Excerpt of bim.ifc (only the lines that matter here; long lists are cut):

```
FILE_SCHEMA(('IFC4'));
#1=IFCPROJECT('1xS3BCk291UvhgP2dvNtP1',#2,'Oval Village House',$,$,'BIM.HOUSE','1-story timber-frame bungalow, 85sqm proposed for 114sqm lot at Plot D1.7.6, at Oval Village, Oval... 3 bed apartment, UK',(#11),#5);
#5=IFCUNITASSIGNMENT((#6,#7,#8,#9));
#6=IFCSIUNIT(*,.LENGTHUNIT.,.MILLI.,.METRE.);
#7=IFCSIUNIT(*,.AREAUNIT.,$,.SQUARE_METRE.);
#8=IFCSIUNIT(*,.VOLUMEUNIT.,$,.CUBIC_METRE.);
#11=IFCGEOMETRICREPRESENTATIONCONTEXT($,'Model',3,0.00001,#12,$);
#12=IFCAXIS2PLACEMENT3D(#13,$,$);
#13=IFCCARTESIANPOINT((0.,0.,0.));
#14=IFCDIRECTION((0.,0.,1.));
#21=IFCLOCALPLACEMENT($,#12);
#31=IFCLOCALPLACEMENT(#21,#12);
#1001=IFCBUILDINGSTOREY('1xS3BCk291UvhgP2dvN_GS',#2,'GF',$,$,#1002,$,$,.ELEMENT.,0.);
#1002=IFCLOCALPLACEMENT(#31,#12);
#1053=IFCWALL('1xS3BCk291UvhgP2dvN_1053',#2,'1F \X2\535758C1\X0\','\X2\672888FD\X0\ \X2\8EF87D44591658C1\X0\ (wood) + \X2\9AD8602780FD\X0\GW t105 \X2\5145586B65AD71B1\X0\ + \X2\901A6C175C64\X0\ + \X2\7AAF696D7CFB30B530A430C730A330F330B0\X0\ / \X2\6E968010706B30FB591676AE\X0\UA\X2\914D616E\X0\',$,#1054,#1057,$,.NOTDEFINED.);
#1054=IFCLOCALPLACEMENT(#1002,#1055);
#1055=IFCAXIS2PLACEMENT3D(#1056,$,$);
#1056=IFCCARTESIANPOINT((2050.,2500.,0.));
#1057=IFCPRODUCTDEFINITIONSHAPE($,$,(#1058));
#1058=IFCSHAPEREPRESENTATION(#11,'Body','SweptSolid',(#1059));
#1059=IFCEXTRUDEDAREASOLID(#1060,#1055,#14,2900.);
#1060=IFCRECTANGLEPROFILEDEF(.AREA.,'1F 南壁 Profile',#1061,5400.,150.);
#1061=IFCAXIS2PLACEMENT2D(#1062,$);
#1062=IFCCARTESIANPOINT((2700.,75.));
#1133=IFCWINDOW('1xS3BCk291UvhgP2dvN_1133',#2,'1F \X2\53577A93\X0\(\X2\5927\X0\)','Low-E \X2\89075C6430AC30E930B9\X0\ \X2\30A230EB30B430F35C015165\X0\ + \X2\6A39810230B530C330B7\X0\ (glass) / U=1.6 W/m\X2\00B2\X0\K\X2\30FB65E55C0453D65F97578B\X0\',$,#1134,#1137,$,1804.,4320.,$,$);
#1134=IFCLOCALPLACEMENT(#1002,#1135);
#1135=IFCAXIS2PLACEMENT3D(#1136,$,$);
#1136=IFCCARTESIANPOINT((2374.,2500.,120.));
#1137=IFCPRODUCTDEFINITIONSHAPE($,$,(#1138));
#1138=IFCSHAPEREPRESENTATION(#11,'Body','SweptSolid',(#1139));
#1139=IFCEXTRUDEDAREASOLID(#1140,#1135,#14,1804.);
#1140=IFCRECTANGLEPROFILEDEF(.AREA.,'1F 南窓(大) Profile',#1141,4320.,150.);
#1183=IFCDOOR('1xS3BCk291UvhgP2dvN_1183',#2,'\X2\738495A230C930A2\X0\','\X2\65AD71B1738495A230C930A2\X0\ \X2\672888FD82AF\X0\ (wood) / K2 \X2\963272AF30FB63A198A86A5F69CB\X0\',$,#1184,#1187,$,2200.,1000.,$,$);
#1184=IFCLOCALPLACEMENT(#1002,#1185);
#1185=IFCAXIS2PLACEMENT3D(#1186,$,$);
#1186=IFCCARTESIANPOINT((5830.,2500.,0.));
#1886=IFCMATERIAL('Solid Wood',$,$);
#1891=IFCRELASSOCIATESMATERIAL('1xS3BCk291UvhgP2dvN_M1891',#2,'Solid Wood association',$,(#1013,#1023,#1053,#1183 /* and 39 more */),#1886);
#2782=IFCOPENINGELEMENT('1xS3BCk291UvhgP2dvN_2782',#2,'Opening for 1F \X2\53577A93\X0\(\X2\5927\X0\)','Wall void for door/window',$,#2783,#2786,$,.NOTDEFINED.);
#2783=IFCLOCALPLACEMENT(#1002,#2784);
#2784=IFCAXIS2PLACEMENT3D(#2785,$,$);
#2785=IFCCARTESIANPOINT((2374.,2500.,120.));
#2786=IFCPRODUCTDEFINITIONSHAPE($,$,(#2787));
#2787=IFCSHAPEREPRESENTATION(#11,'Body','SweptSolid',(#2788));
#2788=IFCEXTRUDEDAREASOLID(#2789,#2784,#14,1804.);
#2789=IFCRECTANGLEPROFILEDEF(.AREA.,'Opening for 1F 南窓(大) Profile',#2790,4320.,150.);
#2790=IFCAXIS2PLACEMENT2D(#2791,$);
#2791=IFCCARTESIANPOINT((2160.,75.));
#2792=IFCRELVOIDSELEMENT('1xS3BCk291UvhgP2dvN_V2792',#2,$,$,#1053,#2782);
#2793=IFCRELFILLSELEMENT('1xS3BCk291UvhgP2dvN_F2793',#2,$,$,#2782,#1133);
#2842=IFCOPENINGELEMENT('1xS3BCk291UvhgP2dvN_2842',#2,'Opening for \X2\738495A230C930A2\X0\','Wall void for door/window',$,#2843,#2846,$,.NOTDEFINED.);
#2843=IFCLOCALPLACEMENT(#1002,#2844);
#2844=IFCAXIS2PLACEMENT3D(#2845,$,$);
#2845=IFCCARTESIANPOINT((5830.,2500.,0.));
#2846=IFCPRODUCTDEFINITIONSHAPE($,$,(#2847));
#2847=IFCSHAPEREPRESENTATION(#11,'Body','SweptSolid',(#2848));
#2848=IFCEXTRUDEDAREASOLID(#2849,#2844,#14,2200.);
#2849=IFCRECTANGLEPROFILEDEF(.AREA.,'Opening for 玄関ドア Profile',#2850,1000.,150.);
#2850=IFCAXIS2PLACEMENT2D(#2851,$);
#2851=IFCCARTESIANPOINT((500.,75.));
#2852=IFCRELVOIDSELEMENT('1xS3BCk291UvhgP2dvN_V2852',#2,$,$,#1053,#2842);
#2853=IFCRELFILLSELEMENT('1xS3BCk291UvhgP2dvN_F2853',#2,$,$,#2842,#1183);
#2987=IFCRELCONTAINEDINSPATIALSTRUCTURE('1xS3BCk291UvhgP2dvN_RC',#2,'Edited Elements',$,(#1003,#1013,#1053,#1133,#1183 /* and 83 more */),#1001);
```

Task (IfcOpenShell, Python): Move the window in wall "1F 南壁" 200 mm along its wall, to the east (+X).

```python
import ifcopenshell
import ifcopenshell.api.geometry
import ifcopenshell.util.placement
import ifcopenshell.util.unit

model = ifcopenshell.open("bim.ifc")
unit_scale = ifcopenshell.util.unit.calculate_unit_scale(model)

window = model.by_guid("1xS3BCk291UvhgP2dvN_1133")
opening = window.FillsVoids[0].RelatingOpeningElement
wall = opening.VoidsElements[0].RelatingBuildingElement

wall_matrix = ifcopenshell.util.placement.get_local_placement(wall.ObjectPlacement)
shift = wall_matrix[:3, 0] * 0.2 / unit_scale
before = ifcopenshell.util.placement.get_local_placement(window.ObjectPlacement)[:3, 3].copy()

# The window is not placed relative to its opening, so move both.
for product in (opening, window):
    matrix = ifcopenshell.util.placement.get_local_placement(product.ObjectPlacement)
    matrix[:3, 3] += shift
    ifcopenshell.api.geometry.edit_object_placement(model, product=product, matrix=matrix, is_si=False)

after = ifcopenshell.util.placement.get_local_placement(window.ObjectPlacement)[:3, 3]
print("window moved by", (after - before).round(3) + 0.0)

model.write("bim_v2.ifc")
```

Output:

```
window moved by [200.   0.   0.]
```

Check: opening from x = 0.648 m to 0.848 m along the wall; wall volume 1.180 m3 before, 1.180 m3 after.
